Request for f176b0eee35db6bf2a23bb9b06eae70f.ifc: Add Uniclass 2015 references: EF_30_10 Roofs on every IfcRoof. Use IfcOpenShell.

First a look at what the model holds.

```python
import ifcopenshell

model = ifcopenshell.open("f176b0eee35db6bf2a23bb9b06eae70f.ifc")
print(model.schema)
print("classifications:", [c.Name for c in model.by_type("IfcClassification")])
for ifc_class in ("IfcDoor", "IfcRoof", "IfcStair", "IfcWall", "IfcWindow"):
    print(ifc_class, len(model.by_type(ifc_class)))
```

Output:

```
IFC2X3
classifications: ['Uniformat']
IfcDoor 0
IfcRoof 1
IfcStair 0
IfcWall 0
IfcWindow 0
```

```python
import ifcopenshell
import ifcopenshell.api.classification

model = ifcopenshell.open("f176b0eee35db6bf2a23bb9b06eae70f.ifc")

# IFC2X3 requires Source and Edition and has no link from the project to the system.
system = model.create_entity("IfcClassification", Source="NBS", Edition="2015", Name="Uniclass 2015")

codes = {
    "IfcRoof": ("EF_30_10", "Roofs"),
}
for ifc_class, (code, name) in codes.items():
    products = model.by_type(ifc_class)
    ifcopenshell.api.classification.add_reference(
        model, products=products, classification=system, identification=code, name=name
    )
    print(code, len(products))

model.write("f176b0eee35db6bf2a23bb9b06eae70f-out.ifc")
```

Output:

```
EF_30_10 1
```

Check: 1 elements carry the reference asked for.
